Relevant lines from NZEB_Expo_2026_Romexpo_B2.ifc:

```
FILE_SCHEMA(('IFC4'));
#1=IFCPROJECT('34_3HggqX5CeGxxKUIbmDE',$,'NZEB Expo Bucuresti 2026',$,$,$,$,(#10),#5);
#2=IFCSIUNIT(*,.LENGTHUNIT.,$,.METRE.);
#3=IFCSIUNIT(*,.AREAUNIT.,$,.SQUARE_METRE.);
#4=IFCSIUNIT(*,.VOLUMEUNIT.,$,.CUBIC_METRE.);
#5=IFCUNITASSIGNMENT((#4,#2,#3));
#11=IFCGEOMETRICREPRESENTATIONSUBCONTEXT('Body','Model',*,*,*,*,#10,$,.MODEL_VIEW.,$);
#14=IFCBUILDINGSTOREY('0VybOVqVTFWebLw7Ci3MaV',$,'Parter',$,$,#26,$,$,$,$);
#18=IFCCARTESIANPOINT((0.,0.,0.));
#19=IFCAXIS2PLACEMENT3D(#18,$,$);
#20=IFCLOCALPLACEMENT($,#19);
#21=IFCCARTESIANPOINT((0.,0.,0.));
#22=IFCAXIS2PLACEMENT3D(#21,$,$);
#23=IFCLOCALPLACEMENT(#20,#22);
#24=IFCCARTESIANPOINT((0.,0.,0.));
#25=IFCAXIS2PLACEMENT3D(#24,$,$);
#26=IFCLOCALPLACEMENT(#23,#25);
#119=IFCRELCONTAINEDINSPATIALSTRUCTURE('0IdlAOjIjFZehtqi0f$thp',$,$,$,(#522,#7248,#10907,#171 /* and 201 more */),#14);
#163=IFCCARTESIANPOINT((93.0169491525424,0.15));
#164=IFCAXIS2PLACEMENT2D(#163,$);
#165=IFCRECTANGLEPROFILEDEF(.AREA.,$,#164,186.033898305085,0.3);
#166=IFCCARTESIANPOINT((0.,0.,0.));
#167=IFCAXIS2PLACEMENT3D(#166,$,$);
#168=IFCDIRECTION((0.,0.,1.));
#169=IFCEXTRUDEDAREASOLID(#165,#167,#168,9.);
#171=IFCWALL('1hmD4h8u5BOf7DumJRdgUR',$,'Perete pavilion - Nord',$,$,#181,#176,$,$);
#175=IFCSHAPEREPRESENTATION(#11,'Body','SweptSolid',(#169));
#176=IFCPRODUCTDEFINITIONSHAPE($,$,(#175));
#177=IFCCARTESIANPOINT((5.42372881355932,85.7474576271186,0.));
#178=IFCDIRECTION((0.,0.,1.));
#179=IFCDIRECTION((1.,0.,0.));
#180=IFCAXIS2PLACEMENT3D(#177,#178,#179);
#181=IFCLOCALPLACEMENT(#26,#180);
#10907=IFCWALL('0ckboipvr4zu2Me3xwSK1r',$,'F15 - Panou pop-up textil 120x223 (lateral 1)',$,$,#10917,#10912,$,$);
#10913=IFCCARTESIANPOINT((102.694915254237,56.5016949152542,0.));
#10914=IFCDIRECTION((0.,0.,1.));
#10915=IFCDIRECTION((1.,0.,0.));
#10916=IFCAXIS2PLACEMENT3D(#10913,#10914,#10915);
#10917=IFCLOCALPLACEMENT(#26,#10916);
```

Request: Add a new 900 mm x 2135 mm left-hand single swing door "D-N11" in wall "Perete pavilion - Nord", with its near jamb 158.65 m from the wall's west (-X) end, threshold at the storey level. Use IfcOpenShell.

```python
import numpy as np
import ifcopenshell
import ifcopenshell.api.feature
import ifcopenshell.api.geometry
import ifcopenshell.api.root
import ifcopenshell.api.spatial
import ifcopenshell.geom
import ifcopenshell.util.element
import ifcopenshell.util.placement
import ifcopenshell.util.representation
import ifcopenshell.util.shape
import ifcopenshell.util.unit

model = ifcopenshell.open("NZEB_Expo_2026_Romexpo_B2.ifc")
unit_scale = ifcopenshell.util.unit.calculate_unit_scale(model)
settings = ifcopenshell.geom.settings()


def volume(element):
    """Net volume in cubic metres, openings subtracted."""
    shape = ifcopenshell.geom.create_shape(settings, element)
    return ifcopenshell.util.shape.get_volume(shape.geometry)


wall = model.by_guid("1hmD4h8u5BOf7DumJRdgUR")
storey = ifcopenshell.util.element.get_container(wall, ifc_class="IfcBuildingStorey")
context = ifcopenshell.util.representation.get_context(model, "Model", "Body", "MODEL_VIEW")
before = volume(wall)

width, height, from_end, sill = 0.9, 2.135, 158.65, 0.0  # metres

# The wall runs along its own X axis, and the end named is its -X end.
wall_shape = ifcopenshell.geom.create_shape(settings, wall)
x, y, z = ifcopenshell.util.shape.get_vertices(wall_shape.geometry).T
start = x.min() + from_end
face, thickness = float(y.min()), float(y.max() - y.min())
wall_matrix = ifcopenshell.util.placement.get_local_placement(wall.ObjectPlacement)
level = ifcopenshell.util.placement.get_local_placement(storey.ObjectPlacement)[2, 3]


def in_wall(x, y):
    """Placement at x, y metres in the wall's axes, at sill height."""
    matrix = wall_matrix.copy()
    matrix[:, 3] = wall_matrix @ np.array([x / unit_scale, y / unit_scale, 0.0, 1.0])
    matrix[2, 3] = level + sill / unit_scale
    return matrix


# Opening: a box that overshoots both wall faces by 50 mm.
opening = ifcopenshell.api.root.create_entity(model, ifc_class="IfcOpeningElement", predefined_type="OPENING")
box = ifcopenshell.api.geometry.add_wall_representation(
    model, context=context, length=width, height=height, thickness=thickness + 0.1
)
ifcopenshell.api.geometry.assign_representation(model, product=opening, representation=box)
ifcopenshell.api.geometry.edit_object_placement(model, product=opening, matrix=in_wall(start, face - 0.05), is_si=False)
ifcopenshell.api.feature.add_feature(model, feature=opening, element=wall)

door = ifcopenshell.api.root.create_entity(model, ifc_class="IfcDoor", name="D-N11", predefined_type="DOOR")
door.OverallWidth, door.OverallHeight = width / unit_scale, height / unit_scale
door.OperationType = "SINGLE_SWING_LEFT"
body = ifcopenshell.api.geometry.add_door_representation(
    model,
    context=context,
    overall_width=door.OverallWidth,
    overall_height=door.OverallHeight,
    operation_type="SINGLE_SWING_LEFT",
    lining_properties={"LiningDepth": thickness / unit_scale, "ThresholdDepth": thickness / unit_scale},
)
ifcopenshell.api.geometry.assign_representation(model, product=door, representation=body)
ifcopenshell.api.spatial.assign_container(model, products=[door], relating_structure=storey)
ifcopenshell.api.feature.add_filling(model, opening=opening, element=door)

# The lining spans the wall, so the door starts at the wall face.
ifcopenshell.api.geometry.edit_object_placement(model, product=door, matrix=in_wall(start, face), is_si=False)

after = volume(wall)

print(f"wall volume {before:.3f} -> {after:.3f} m3")

model.write("NZEB_Expo_2026_Romexpo_B2_edited.ifc")
```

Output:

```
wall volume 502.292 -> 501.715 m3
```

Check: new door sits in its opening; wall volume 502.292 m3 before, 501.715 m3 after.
